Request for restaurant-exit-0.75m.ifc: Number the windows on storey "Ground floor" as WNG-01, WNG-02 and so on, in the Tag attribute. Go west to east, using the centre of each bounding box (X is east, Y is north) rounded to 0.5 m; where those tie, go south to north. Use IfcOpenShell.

First a look at what the model holds.

```python
import ifcopenshell
import ifcopenshell.util.element
import ifcopenshell.util.placement

model = ifcopenshell.open("restaurant-exit-0.75m.ifc")
print(model.schema)
storey = next(s for s in model.by_type("IfcBuildingStorey") if s.Name == "Ground floor")
windows = [e for e in ifcopenshell.util.element.get_decomposition(storey) if e.is_a("IfcWindow")]
for e in sorted(windows, key=lambda e: e.id()):
    origin = ifcopenshell.util.placement.get_local_placement(e.ObjectPlacement)[:3, 3]
    print(e.id(), e.Tag, e.Name, origin.round(2) + 0.0, sep=" | ")
```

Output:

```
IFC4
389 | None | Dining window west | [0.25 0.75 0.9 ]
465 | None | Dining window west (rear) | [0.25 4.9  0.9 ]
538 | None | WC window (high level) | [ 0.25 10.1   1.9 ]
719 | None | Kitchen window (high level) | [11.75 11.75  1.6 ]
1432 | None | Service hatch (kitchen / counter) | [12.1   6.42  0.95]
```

```python
import ifcopenshell
import ifcopenshell.geom
import ifcopenshell.util.element
import ifcopenshell.util.shape

model = ifcopenshell.open("restaurant-exit-0.75m.ifc")
settings = ifcopenshell.geom.settings()
settings.set("use-world-coords", True)


def centre(element):
    shape = ifcopenshell.geom.create_shape(settings, element)
    return ifcopenshell.util.shape.get_bbox_centroid(shape.geometry)


storey = next(s for s in model.by_type("IfcBuildingStorey") if s.Name == "Ground floor")
windows = [e for e in ifcopenshell.util.element.get_decomposition(storey) if e.is_a("IfcWindow")]

# Insertion points can sit at a corner or the storey origin, so sort by the geometry (in metres).
centres = {e: centre(e) for e in windows}
windows.sort(key=lambda e: (round(centres[e][0] / 0.5), centres[e][1]))

for i, e in enumerate(windows, start=1):
    number = f"WNG-{i:02d}"
    e.Tag = number
    print(e.id(), number)

model.write("restaurant-exit-0.75m_updated.ifc")
```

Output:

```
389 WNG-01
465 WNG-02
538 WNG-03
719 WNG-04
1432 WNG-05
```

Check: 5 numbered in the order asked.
